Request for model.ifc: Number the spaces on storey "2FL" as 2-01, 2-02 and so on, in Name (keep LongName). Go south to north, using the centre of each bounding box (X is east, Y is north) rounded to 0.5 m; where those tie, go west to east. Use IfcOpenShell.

First a look at what the model holds.

```python
import ifcopenshell
import ifcopenshell.util.element
import ifcopenshell.util.placement

model = ifcopenshell.open("model.ifc")
print(model.schema)
storey = next(s for s in model.by_type("IfcBuildingStorey") if s.Name == "2FL")
spaces = [e for e in ifcopenshell.util.element.get_decomposition(storey) if e.is_a("IfcSpace")]
for e in sorted(spaces, key=lambda e: e.id()):
    origin = ifcopenshell.util.placement.get_local_placement(e.ObjectPlacement)[:3, 3]
    print(e.id(), e.Name, e.LongName, origin.round(2) + 0.0, sep=" | ")
```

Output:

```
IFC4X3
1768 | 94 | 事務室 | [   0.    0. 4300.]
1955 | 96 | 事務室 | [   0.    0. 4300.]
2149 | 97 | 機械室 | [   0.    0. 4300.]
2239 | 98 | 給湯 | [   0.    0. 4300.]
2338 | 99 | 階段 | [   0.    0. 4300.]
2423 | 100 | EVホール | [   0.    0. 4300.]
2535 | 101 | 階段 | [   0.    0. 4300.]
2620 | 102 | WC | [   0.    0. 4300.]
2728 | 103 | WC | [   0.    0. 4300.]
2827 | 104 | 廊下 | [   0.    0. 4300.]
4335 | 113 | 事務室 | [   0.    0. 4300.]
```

```python
import ifcopenshell
import ifcopenshell.geom
import ifcopenshell.util.element
import ifcopenshell.util.shape

model = ifcopenshell.open("model.ifc")
settings = ifcopenshell.geom.settings()
settings.set("use-world-coords", True)


def centre(element):
    shape = ifcopenshell.geom.create_shape(settings, element)
    return ifcopenshell.util.shape.get_bbox_centroid(shape.geometry)


storey = next(s for s in model.by_type("IfcBuildingStorey") if s.Name == "2FL")
spaces = [e for e in ifcopenshell.util.element.get_decomposition(storey) if e.is_a("IfcSpace")]

# Insertion points can sit at a corner or the storey origin, so sort by the geometry (in metres).
centres = {e: centre(e) for e in spaces}
spaces.sort(key=lambda e: (round(centres[e][1] / 0.5), centres[e][0]))

for i, e in enumerate(spaces, start=1):
    number = f"2-{i:02d}"
    e.Name = number
    print(e.id(), number)

model.write("model_rev.ifc")
```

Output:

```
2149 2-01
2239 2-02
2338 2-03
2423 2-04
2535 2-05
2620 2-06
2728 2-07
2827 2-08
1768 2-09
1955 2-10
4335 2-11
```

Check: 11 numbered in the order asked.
